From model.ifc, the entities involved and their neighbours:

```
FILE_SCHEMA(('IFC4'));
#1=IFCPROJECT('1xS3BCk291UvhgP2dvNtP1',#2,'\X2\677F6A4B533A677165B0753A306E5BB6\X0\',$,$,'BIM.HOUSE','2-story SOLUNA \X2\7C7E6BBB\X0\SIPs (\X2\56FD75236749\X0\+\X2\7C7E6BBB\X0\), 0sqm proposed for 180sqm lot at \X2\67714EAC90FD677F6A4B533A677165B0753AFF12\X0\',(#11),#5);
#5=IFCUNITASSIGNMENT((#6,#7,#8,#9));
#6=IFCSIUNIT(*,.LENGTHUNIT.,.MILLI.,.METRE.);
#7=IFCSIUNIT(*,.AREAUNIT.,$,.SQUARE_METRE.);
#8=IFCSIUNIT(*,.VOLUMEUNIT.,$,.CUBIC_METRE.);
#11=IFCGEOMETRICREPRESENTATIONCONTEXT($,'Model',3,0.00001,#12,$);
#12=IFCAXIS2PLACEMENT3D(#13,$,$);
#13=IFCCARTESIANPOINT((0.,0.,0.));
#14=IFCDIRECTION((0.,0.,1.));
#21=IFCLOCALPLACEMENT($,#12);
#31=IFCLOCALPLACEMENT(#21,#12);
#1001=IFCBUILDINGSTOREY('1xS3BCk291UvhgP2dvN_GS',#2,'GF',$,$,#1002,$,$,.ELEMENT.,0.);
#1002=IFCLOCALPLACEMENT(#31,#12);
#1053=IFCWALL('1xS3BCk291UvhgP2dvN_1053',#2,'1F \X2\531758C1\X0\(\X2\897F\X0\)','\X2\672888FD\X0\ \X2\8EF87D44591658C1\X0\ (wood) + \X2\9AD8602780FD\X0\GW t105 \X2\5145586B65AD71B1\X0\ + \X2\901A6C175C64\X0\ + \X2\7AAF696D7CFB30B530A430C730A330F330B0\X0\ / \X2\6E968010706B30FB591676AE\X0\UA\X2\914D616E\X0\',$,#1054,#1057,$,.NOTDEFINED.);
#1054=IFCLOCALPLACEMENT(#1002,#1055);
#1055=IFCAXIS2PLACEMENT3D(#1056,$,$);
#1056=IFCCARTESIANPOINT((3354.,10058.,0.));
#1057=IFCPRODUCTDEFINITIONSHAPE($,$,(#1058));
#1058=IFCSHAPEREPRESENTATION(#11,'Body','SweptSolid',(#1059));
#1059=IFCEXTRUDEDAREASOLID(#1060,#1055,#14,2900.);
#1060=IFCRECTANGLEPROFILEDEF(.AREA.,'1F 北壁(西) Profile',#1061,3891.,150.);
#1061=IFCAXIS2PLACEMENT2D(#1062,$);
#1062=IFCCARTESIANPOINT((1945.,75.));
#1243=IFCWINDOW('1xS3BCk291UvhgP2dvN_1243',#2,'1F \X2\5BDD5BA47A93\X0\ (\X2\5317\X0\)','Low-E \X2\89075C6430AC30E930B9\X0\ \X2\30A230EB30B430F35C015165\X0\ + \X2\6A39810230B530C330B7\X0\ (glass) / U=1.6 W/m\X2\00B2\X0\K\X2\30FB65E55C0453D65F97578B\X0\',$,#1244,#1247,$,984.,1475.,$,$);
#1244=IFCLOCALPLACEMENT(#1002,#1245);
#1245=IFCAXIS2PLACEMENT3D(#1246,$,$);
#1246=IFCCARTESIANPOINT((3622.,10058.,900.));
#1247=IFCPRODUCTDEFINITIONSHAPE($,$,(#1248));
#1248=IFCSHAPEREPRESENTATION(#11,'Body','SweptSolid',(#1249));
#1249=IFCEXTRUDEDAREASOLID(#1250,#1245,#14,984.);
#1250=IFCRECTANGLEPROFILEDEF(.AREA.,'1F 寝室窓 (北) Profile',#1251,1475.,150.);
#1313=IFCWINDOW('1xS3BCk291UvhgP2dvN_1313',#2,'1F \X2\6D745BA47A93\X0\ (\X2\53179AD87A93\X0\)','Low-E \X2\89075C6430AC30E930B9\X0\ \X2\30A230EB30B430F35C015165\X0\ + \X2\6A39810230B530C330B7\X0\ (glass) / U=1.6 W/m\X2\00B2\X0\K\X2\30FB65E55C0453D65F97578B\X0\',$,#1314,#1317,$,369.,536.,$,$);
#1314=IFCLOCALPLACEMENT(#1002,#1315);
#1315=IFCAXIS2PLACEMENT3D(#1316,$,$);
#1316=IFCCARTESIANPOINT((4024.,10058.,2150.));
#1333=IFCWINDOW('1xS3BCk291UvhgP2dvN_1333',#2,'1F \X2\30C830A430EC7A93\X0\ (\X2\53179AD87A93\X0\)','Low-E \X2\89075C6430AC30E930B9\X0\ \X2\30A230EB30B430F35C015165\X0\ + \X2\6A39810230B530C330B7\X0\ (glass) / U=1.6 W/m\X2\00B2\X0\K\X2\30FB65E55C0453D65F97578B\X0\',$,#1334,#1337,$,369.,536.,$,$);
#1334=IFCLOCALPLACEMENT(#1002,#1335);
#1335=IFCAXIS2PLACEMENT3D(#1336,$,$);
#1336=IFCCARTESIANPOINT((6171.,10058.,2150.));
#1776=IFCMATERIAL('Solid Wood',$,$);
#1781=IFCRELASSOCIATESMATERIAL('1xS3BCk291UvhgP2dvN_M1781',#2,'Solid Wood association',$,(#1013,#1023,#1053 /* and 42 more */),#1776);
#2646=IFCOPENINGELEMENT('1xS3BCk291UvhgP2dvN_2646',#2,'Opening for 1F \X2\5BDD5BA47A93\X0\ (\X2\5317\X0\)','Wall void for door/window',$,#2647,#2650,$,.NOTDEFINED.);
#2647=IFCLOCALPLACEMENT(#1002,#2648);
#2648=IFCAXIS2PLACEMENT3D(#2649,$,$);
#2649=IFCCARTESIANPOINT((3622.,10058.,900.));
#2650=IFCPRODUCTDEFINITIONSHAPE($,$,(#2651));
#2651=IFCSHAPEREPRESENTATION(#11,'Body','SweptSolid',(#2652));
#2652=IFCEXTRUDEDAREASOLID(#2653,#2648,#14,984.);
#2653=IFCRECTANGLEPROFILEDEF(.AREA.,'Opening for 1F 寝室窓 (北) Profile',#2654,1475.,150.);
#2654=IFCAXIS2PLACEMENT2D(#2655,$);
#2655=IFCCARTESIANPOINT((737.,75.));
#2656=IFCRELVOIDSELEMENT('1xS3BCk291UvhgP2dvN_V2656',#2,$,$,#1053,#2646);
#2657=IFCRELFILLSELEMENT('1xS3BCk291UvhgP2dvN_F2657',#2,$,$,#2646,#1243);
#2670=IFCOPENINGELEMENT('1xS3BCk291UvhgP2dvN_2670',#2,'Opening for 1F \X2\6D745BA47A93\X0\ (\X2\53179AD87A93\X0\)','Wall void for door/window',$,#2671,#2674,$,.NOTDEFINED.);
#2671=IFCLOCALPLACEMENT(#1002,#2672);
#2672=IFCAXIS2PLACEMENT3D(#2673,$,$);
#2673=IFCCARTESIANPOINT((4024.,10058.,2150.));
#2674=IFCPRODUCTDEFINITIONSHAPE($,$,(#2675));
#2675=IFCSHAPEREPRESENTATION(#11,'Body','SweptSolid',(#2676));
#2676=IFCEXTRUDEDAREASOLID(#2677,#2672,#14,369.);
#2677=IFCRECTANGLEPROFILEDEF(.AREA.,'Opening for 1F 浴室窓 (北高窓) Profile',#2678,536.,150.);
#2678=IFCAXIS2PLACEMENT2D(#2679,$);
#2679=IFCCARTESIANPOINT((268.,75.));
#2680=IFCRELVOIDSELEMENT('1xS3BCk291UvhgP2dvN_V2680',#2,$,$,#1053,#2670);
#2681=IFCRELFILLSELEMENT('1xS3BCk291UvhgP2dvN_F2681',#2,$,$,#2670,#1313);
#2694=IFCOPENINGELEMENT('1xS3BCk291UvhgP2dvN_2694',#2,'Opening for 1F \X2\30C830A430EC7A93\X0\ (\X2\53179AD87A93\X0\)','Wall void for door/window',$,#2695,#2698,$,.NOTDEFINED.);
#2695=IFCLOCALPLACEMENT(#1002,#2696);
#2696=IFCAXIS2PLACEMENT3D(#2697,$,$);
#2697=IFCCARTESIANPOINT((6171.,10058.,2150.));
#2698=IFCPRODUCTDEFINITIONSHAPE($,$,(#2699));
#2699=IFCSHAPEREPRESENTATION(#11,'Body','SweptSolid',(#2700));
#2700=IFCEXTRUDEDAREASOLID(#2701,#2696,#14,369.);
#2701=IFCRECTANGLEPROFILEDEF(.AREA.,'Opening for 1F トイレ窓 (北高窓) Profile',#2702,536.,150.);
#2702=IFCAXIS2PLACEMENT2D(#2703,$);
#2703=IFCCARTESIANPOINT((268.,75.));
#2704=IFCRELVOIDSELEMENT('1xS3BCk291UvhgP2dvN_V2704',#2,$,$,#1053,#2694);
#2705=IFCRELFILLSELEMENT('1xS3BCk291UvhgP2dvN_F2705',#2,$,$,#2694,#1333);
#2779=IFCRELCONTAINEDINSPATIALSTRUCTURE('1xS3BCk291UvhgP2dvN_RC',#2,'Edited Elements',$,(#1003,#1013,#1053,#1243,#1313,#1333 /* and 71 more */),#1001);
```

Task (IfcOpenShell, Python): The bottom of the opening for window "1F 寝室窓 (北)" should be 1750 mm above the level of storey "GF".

```python
import numpy as np
import ifcopenshell
import ifcopenshell.api.geometry
import ifcopenshell.geom
import ifcopenshell.util.element
import ifcopenshell.util.placement
import ifcopenshell.util.shape
import ifcopenshell.util.unit

model = ifcopenshell.open("model.ifc")
unit_scale = ifcopenshell.util.unit.calculate_unit_scale(model)

window = model.by_guid("1xS3BCk291UvhgP2dvN_1243")
opening = window.FillsVoids[0].RelatingOpeningElement
storey = ifcopenshell.util.element.get_container(window, ifc_class="IfcBuildingStorey")
level = ifcopenshell.util.placement.get_local_placement(storey.ObjectPlacement)[2, 3]

# The opening's origin need not be at the sill, so measure its lowest point.
shape = ifcopenshell.geom.create_shape(ifcopenshell.geom.settings(), opening)
bottom = ifcopenshell.util.shape.get_shape_bottom_elevation(shape, shape.geometry) / unit_scale
dz = level + 1750.0 - bottom

shift = np.array([0.0, 0.0, dz])
# The window is not placed relative to its opening, so move both.
for product in (opening, window):
    matrix = ifcopenshell.util.placement.get_local_placement(product.ObjectPlacement)
    matrix[:3, 3] += shift
    ifcopenshell.api.geometry.edit_object_placement(model, product=product, matrix=matrix, is_si=False)

print(f"moved by {dz * unit_scale:+.3f} m")

model.write("model-out.ifc")
```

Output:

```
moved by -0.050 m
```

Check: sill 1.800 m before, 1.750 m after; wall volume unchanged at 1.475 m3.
